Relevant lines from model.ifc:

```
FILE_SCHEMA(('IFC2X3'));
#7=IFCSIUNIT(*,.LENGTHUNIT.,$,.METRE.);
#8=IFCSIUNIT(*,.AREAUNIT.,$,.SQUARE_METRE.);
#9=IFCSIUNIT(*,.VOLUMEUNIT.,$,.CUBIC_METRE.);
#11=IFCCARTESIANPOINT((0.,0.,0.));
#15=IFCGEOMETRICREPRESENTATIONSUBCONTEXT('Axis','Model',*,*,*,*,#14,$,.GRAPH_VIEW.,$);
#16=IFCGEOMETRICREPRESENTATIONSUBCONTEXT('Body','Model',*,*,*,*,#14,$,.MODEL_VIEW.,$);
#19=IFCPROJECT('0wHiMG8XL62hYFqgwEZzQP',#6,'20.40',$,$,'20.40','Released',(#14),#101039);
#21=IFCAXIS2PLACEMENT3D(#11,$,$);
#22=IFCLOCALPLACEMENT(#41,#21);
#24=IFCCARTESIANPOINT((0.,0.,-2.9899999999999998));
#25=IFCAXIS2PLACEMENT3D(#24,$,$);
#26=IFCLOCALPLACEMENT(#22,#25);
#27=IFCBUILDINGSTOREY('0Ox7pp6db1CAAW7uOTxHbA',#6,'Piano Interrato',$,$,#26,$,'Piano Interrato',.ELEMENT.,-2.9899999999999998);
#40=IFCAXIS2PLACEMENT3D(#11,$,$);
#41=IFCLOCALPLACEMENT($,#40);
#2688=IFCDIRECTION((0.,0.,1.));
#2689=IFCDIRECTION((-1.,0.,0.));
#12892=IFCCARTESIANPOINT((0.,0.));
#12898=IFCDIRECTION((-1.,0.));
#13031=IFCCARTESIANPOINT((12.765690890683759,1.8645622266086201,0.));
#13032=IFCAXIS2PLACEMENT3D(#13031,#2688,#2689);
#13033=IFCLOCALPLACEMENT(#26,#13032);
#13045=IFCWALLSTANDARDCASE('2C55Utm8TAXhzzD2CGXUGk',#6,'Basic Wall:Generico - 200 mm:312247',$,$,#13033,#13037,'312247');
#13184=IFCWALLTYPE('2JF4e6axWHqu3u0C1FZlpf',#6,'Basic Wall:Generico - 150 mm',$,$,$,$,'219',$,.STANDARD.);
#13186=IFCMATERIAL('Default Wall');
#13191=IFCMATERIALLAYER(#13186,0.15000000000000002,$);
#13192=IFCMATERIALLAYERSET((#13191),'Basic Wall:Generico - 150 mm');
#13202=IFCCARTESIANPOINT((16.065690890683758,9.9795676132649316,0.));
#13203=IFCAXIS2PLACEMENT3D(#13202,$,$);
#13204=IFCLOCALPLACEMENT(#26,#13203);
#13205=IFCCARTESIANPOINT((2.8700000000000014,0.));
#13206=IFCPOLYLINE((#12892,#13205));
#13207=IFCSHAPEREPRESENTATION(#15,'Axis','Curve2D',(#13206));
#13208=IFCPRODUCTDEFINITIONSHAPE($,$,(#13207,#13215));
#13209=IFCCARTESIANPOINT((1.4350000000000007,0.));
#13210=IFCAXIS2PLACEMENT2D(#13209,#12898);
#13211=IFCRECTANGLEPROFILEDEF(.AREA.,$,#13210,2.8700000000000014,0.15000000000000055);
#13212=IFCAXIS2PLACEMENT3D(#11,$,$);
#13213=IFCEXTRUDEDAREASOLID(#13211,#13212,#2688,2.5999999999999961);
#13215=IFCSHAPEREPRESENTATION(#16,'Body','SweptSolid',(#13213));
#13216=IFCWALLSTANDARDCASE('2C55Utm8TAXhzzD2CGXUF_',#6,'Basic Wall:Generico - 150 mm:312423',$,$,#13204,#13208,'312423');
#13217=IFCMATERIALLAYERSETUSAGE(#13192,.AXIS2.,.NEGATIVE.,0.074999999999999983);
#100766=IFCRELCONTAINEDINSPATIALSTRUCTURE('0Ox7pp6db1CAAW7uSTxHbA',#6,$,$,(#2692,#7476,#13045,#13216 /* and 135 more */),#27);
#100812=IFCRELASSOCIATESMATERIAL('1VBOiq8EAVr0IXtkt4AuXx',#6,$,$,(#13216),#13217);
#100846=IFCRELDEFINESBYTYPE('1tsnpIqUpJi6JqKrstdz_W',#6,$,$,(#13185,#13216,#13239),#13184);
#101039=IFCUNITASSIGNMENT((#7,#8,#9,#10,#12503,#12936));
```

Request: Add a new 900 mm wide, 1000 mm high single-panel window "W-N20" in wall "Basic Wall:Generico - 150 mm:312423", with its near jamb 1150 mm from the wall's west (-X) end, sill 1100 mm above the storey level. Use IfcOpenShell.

```python
import numpy as np
import ifcopenshell
import ifcopenshell.api.feature
import ifcopenshell.api.geometry
import ifcopenshell.api.root
import ifcopenshell.api.spatial
import ifcopenshell.api.type
import ifcopenshell.geom
import ifcopenshell.util.element
import ifcopenshell.util.placement
import ifcopenshell.util.representation
import ifcopenshell.util.shape
import ifcopenshell.util.unit

model = ifcopenshell.open("model.ifc")
unit_scale = ifcopenshell.util.unit.calculate_unit_scale(model)
settings = ifcopenshell.geom.settings()


def volume(element):
    """Net volume in cubic metres, openings subtracted."""
    shape = ifcopenshell.geom.create_shape(settings, element)
    return ifcopenshell.util.shape.get_volume(shape.geometry)


wall = model.by_id(13216)
storey = ifcopenshell.util.element.get_container(wall, ifc_class="IfcBuildingStorey")
context = ifcopenshell.util.representation.get_context(model, "Model", "Body", "MODEL_VIEW")
before = volume(wall)

width, height, from_end, sill = 0.9, 1, 1.15, 1.1  # metres

# The wall runs along its own X axis, and the end named is its -X end.
wall_shape = ifcopenshell.geom.create_shape(settings, wall)
x, y, z = ifcopenshell.util.shape.get_vertices(wall_shape.geometry).T
start = x.min() + from_end
face, thickness = float(y.min()), float(y.max() - y.min())
wall_matrix = ifcopenshell.util.placement.get_local_placement(wall.ObjectPlacement)
level = ifcopenshell.util.placement.get_local_placement(storey.ObjectPlacement)[2, 3]


def in_wall(x, y):
    """Placement at x, y metres in the wall's axes, at sill height."""
    matrix = wall_matrix.copy()
    matrix[:, 3] = wall_matrix @ np.array([x / unit_scale, y / unit_scale, 0.0, 1.0])
    matrix[2, 3] = level + sill / unit_scale
    return matrix


# Opening: a box that overshoots both wall faces by 50 mm.
opening = ifcopenshell.api.root.create_entity(model, ifc_class="IfcOpeningElement")
box = ifcopenshell.api.geometry.add_wall_representation(
    model, context=context, length=width, height=height, thickness=thickness + 0.1
)
ifcopenshell.api.geometry.assign_representation(model, product=opening, representation=box)
ifcopenshell.api.geometry.edit_object_placement(model, product=opening, matrix=in_wall(start, face - 0.05), is_si=False)
ifcopenshell.api.feature.add_feature(model, feature=opening, element=wall)

window = ifcopenshell.api.root.create_entity(model, ifc_class="IfcWindow", name="W-N20")
window.OverallWidth, window.OverallHeight = width / unit_scale, height / unit_scale
body = ifcopenshell.api.geometry.add_window_representation(
    model,
    context=context,
    overall_width=window.OverallWidth,
    overall_height=window.OverallHeight,
    partition_type="SINGLE_PANEL",
)
ifcopenshell.api.geometry.assign_representation(model, product=window, representation=body)
ifcopenshell.api.spatial.assign_container(model, products=[window], relating_structure=storey)
fills = ifcopenshell.api.feature.add_filling(model, opening=opening, element=window)
fills.OwnerHistory = window.OwnerHistory  # required in IFC2X3

# IFC2X3 keeps the operation on the window style.
style = ifcopenshell.api.root.create_entity(model, ifc_class="IfcWindowStyle", name="W-N20")
style.OperationType, style.ConstructionType = "SINGLE_PANEL", "NOTDEFINED"
style.ParameterTakesPrecedence = style.Sizeable = False
ifcopenshell.api.type.assign_type(model, related_objects=[window], relating_type=style)

# Centre the window in the wall's thickness.
ifcopenshell.api.geometry.edit_object_placement(model, product=window, matrix=in_wall(start, face), is_si=False)
window_shape = ifcopenshell.geom.create_shape(settings, window)
depth = ifcopenshell.util.shape.get_vertices(window_shape.geometry)[:, 1]
offset = face + thickness / 2 - (depth.min() + depth.max()) / 2
ifcopenshell.api.geometry.edit_object_placement(model, product=window, matrix=in_wall(start, offset), is_si=False)

after = volume(wall)

print(f"wall volume {before:.3f} -> {after:.3f} m3")

model.write("model_rev.ifc")
```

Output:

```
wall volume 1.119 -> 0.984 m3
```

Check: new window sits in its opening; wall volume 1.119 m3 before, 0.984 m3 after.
